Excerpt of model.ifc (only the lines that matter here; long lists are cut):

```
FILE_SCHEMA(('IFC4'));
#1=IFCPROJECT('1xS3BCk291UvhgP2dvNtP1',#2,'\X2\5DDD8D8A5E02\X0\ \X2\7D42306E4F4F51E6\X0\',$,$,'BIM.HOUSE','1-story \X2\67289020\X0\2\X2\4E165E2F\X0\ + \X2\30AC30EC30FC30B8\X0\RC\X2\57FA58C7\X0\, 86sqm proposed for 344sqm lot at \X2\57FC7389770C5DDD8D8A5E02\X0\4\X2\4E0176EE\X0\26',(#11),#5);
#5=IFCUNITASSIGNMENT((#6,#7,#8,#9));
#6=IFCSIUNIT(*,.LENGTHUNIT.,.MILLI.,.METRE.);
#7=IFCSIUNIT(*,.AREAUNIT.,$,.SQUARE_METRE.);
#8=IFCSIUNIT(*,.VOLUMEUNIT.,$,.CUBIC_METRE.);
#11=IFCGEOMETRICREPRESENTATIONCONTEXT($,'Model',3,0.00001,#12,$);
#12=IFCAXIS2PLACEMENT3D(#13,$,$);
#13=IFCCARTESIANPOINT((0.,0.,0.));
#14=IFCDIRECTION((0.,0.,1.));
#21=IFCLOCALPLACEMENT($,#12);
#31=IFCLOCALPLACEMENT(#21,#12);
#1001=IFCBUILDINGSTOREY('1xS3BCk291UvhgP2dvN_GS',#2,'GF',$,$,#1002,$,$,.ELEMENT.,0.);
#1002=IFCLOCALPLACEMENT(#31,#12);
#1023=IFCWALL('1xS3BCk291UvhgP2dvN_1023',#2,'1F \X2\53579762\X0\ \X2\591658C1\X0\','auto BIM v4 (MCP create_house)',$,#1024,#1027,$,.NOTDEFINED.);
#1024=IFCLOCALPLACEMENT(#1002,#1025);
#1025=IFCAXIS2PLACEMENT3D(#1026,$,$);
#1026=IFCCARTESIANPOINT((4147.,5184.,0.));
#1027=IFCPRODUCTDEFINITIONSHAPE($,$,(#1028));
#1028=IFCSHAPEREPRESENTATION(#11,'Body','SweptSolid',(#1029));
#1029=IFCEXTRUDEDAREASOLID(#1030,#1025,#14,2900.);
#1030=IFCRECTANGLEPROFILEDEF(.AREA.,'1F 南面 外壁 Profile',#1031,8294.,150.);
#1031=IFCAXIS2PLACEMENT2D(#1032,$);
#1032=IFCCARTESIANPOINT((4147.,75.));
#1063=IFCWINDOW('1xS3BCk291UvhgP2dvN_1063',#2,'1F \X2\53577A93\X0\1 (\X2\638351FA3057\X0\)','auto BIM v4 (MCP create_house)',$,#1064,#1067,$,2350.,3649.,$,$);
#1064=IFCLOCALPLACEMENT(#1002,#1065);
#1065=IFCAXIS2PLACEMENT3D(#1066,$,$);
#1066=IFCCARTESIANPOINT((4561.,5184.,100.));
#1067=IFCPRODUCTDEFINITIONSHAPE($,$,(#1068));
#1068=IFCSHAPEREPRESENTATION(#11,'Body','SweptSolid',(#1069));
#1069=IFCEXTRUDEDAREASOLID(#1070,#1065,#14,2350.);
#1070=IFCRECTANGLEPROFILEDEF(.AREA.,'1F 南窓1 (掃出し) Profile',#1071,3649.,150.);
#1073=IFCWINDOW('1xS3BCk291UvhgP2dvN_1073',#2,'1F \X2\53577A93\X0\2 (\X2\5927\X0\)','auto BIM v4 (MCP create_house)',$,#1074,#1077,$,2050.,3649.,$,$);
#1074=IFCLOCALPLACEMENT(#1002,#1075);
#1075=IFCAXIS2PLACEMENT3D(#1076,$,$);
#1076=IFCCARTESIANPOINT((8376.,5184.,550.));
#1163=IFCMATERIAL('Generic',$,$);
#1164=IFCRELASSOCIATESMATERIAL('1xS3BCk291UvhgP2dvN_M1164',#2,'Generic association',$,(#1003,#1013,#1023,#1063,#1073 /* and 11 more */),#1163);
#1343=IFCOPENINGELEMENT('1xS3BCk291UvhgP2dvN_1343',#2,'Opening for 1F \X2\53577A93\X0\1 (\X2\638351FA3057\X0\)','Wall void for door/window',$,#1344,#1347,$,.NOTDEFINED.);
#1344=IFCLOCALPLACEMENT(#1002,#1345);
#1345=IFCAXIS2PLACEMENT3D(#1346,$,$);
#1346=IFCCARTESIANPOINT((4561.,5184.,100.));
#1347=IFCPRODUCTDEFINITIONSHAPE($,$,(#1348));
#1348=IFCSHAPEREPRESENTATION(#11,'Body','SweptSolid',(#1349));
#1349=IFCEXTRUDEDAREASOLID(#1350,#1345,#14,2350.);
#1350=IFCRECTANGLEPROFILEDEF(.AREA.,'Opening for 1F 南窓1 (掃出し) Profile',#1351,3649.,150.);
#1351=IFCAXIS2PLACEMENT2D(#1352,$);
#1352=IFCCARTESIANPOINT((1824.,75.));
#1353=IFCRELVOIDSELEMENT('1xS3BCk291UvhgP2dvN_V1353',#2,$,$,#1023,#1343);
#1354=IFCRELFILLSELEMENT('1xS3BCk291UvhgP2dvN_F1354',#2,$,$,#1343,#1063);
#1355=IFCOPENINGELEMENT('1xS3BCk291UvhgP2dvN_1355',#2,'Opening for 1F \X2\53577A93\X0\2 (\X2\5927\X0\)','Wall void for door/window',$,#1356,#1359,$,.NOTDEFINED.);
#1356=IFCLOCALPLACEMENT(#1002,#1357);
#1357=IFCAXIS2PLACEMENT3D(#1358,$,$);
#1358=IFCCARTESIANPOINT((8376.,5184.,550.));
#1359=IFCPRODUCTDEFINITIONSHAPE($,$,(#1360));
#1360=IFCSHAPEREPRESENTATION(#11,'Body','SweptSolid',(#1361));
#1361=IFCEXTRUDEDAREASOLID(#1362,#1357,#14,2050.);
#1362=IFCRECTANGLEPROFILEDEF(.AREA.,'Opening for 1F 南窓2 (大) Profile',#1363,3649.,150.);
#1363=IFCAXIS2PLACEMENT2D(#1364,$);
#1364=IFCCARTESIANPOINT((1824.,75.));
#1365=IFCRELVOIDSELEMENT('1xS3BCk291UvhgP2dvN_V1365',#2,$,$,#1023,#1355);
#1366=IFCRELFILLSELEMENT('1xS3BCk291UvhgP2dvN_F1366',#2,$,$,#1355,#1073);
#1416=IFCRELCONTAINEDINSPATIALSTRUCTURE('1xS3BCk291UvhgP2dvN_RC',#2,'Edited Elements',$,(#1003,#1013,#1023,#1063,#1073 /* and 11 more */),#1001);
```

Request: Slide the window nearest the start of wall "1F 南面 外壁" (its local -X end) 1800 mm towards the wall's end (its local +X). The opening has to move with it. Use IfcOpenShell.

```python
import ifcopenshell
import ifcopenshell.api.geometry
import ifcopenshell.util.placement
import ifcopenshell.util.unit

model = ifcopenshell.open("model.ifc")
unit_scale = ifcopenshell.util.unit.calculate_unit_scale(model)

window = model.by_id(1063)
opening = window.FillsVoids[0].RelatingOpeningElement
wall = opening.VoidsElements[0].RelatingBuildingElement

wall_matrix = ifcopenshell.util.placement.get_local_placement(wall.ObjectPlacement)
shift = wall_matrix[:3, 0] * 1.8 / unit_scale
before = ifcopenshell.util.placement.get_local_placement(window.ObjectPlacement)[:3, 3].copy()

# The window is not placed relative to its opening, so move both.
for product in (opening, window):
    matrix = ifcopenshell.util.placement.get_local_placement(product.ObjectPlacement)
    matrix[:3, 3] += shift
    ifcopenshell.api.geometry.edit_object_placement(model, product=product, matrix=matrix, is_si=False)

after = ifcopenshell.util.placement.get_local_placement(window.ObjectPlacement)[:3, 3]
print("window moved by", (after - before).round(3) + 0.0)

model.write("model_updated.ifc")
```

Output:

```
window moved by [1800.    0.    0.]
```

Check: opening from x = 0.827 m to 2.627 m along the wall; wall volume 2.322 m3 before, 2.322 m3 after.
